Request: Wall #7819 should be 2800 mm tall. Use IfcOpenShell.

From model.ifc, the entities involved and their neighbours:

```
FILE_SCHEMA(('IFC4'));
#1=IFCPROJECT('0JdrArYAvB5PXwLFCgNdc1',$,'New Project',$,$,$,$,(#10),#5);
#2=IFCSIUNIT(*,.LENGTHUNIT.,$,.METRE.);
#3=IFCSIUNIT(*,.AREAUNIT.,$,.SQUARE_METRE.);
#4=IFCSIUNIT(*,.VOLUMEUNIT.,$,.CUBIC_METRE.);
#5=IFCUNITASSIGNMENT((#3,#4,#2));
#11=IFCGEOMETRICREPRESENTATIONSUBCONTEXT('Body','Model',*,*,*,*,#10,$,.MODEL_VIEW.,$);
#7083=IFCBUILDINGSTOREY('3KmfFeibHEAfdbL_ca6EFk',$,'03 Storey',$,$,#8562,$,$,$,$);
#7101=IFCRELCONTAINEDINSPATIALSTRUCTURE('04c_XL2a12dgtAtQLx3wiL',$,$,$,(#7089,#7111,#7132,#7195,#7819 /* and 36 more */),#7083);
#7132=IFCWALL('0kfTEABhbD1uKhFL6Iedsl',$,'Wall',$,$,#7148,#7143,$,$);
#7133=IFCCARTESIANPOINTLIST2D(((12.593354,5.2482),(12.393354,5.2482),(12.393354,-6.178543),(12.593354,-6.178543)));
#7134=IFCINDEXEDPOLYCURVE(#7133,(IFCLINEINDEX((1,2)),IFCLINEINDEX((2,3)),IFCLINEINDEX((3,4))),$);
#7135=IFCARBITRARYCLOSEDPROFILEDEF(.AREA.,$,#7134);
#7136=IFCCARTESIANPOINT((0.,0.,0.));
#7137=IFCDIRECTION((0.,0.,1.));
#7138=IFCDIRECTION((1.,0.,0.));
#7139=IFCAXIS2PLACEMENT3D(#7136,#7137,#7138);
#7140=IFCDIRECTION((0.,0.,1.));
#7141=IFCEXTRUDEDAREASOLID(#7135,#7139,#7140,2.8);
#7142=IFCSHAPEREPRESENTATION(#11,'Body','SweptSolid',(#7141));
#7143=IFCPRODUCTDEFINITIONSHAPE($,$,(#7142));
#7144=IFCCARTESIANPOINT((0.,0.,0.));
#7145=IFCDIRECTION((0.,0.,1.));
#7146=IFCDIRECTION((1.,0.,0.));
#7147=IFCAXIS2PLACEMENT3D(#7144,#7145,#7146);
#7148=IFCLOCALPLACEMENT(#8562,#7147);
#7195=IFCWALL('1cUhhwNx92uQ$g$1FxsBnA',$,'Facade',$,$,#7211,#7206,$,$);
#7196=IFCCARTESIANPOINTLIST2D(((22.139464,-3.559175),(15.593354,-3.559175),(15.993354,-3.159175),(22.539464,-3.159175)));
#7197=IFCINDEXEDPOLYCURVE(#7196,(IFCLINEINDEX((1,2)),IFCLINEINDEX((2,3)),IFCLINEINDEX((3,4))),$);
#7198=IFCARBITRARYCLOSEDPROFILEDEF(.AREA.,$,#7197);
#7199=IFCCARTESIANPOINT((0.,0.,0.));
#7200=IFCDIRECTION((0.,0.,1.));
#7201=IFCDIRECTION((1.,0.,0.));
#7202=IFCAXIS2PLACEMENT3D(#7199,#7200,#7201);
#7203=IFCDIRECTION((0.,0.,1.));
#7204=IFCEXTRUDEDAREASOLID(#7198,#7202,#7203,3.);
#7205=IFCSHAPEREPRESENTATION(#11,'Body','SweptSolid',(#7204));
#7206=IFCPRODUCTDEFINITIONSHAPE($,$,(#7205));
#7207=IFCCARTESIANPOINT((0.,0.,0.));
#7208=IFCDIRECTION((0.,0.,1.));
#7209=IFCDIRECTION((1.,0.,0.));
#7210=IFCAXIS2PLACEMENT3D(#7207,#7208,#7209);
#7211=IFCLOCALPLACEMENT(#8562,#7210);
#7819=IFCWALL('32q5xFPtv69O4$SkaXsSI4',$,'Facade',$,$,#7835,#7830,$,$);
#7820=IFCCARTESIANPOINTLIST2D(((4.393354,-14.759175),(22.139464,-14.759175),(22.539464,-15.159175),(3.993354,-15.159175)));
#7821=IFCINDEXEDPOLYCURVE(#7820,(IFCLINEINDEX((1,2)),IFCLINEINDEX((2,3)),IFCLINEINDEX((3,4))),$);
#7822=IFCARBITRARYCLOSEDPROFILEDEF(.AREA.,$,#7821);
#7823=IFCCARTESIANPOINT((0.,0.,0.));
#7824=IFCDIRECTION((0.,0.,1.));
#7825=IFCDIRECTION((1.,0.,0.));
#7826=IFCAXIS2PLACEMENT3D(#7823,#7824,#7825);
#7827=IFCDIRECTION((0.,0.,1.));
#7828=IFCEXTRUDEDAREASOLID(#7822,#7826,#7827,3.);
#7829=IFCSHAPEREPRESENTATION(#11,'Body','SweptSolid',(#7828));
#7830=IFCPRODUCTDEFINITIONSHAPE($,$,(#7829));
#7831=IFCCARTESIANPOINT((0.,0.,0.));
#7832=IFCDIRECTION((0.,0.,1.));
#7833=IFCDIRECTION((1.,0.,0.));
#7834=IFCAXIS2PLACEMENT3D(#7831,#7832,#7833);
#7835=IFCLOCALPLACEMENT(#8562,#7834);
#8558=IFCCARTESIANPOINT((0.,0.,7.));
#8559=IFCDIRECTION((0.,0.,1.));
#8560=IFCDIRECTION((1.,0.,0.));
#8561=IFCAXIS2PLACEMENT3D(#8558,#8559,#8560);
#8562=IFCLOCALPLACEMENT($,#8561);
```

```python
import ifcopenshell
import ifcopenshell.geom
import ifcopenshell.util.representation
import ifcopenshell.util.shape
import ifcopenshell.util.unit

model = ifcopenshell.open("model.ifc")
unit_scale = ifcopenshell.util.unit.calculate_unit_scale(model)
settings = ifcopenshell.geom.settings()


def volume(element):
    """Net volume in cubic metres, openings subtracted."""
    shape = ifcopenshell.geom.create_shape(settings, element)
    return ifcopenshell.util.shape.get_volume(shape.geometry)


wall = model.by_guid("32q5xFPtv69O4$SkaXsSI4")
before = volume(wall)

body = ifcopenshell.util.representation.get_representation(wall, "Model", "Body")
solid = body.Items[0]
old_height = solid.Depth
solid.Depth = 2.8 / unit_scale
after = volume(wall)

print(f"height {old_height:g} -> {solid.Depth:g}, volume {before:.3f} -> {after:.3f} m3")

model.write("model_updated.ifc")
```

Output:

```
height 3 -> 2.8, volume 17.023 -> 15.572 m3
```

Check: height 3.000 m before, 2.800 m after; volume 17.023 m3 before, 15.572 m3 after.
